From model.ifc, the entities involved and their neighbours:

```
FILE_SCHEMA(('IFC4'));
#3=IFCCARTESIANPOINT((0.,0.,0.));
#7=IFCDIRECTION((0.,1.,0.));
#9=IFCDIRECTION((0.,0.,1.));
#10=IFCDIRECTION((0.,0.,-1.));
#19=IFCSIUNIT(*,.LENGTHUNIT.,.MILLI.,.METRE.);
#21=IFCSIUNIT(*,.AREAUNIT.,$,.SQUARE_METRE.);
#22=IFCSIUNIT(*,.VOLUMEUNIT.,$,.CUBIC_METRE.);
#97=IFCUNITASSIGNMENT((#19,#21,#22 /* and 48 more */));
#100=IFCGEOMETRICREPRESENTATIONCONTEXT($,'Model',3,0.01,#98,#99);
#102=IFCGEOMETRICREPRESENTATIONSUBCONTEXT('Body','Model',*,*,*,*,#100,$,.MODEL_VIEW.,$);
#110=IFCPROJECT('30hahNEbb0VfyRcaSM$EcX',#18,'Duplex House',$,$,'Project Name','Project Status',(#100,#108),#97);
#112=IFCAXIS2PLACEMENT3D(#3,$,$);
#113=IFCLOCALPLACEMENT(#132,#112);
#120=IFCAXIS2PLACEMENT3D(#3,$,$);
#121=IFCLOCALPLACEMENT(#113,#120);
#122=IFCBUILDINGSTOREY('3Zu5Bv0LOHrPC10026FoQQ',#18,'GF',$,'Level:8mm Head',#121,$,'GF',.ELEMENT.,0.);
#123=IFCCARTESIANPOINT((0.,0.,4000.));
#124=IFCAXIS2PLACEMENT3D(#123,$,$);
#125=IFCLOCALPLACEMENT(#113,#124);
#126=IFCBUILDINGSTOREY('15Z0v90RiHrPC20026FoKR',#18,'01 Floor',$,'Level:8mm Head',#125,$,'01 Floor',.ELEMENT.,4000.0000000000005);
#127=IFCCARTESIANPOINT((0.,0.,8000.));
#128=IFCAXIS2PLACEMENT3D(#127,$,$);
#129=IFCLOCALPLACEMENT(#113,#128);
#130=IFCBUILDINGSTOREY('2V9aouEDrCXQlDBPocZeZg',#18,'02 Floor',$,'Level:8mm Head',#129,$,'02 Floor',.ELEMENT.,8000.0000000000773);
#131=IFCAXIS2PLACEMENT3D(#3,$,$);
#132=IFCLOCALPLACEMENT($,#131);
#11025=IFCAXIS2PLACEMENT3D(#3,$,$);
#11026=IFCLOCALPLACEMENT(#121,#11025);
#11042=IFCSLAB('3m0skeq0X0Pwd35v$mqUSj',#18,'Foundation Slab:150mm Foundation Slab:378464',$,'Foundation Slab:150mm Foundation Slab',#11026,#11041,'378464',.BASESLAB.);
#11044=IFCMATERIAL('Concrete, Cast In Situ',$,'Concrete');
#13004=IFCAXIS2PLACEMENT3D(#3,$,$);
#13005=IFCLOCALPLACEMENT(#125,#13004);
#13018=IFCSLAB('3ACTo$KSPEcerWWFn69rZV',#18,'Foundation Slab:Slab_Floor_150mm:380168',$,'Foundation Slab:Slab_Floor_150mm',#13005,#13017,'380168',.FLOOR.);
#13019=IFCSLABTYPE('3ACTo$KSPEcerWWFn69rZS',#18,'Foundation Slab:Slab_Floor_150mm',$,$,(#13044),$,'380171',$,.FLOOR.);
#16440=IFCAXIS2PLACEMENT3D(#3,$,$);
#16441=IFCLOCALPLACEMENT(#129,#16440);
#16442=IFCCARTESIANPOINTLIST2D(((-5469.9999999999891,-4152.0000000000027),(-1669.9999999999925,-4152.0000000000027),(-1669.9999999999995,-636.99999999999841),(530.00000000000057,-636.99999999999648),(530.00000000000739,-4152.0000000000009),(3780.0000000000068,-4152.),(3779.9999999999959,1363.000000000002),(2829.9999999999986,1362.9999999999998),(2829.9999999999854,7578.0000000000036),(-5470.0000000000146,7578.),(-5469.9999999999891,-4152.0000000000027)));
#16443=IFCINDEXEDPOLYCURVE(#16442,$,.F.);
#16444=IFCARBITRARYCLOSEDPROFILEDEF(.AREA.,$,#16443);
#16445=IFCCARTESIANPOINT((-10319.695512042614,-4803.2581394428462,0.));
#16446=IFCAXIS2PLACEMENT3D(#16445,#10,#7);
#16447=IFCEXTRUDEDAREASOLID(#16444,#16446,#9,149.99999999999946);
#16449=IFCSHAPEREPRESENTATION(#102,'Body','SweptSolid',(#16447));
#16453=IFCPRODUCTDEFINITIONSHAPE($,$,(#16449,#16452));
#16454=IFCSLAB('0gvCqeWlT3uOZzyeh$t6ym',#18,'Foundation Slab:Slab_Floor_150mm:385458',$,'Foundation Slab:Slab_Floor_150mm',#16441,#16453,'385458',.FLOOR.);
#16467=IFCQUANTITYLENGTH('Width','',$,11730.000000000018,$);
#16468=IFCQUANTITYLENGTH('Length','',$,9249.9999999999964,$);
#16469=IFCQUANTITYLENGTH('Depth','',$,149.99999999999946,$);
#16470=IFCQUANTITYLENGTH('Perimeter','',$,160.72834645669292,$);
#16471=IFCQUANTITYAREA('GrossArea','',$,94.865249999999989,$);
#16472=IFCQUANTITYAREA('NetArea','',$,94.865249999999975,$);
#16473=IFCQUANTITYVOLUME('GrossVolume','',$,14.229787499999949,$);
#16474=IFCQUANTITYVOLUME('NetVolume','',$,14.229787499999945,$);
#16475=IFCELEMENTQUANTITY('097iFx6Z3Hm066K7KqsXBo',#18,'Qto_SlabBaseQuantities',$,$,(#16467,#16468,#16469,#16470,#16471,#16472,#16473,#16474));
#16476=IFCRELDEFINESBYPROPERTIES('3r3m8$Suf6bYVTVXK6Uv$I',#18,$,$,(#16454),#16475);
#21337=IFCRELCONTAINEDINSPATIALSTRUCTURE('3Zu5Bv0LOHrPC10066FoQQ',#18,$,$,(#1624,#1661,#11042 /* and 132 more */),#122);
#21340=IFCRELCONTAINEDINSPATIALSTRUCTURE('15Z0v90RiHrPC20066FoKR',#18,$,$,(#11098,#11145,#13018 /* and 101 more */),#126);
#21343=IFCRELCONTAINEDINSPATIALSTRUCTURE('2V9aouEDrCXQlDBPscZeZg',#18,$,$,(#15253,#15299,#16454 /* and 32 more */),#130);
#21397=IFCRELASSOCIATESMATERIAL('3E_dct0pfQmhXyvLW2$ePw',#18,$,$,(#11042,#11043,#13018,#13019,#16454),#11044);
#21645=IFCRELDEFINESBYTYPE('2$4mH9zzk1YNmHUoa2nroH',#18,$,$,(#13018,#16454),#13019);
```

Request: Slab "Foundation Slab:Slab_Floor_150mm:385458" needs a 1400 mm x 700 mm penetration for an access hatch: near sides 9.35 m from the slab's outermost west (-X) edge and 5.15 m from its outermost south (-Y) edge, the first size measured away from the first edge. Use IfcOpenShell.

```python
import numpy as np
import ifcopenshell
import ifcopenshell.api.feature
import ifcopenshell.api.geometry
import ifcopenshell.api.pset
import ifcopenshell.api.root
import ifcopenshell.geom
import ifcopenshell.util.element
import ifcopenshell.util.placement
import ifcopenshell.util.representation
import ifcopenshell.util.shape
import ifcopenshell.util.unit

model = ifcopenshell.open("model.ifc")
unit_scale = ifcopenshell.util.unit.calculate_unit_scale(model)
area_scale = ifcopenshell.util.unit.calculate_unit_scale(model, "AREAUNIT")
volume_scale = ifcopenshell.util.unit.calculate_unit_scale(model, "VOLUMEUNIT")
settings = ifcopenshell.geom.settings()


def volume(element):
    """Net volume in cubic metres, openings subtracted."""
    shape = ifcopenshell.geom.create_shape(settings, element)
    return ifcopenshell.util.shape.get_volume(shape.geometry)


slab = model.by_guid("0gvCqeWlT3uOZzyeh$t6ym")
before = volume(slab)

# Extent in the slab's own axes, in metres. The edges named are its -X and -Y sides.
slab_shape = ifcopenshell.geom.create_shape(settings, slab)
vertices = ifcopenshell.util.shape.get_vertices(slab_shape.geometry)
x_min, y_min, bottom = vertices.min(axis=0)
top = vertices[:, 2].max()

opening = ifcopenshell.api.root.create_entity(model, ifc_class="IfcOpeningElement", name="Access hatch opening", predefined_type="OPENING")
context = ifcopenshell.util.representation.get_context(model, "Model", "Body", "MODEL_VIEW")
width, depth = 1.4, 0.7
outline = [(0.0, 0.0), (width, 0.0), (width, depth), (0.0, depth), (0.0, 0.0)]
# Overshoot both faces by 50 mm so the cut is clean.
shape = ifcopenshell.api.geometry.add_slab_representation(
    model, context=context, depth=top - bottom + 0.1, polyline=outline
)
ifcopenshell.api.geometry.assign_representation(model, product=opening, representation=shape)

matrix = ifcopenshell.util.placement.get_local_placement(slab.ObjectPlacement)
matrix[:, 3] = matrix @ np.append(np.array([x_min + 9.35, y_min + 5.15, bottom - 0.05]) / unit_scale, 1.0)
ifcopenshell.api.geometry.edit_object_placement(model, product=opening, matrix=matrix, is_si=False)
ifcopenshell.api.feature.add_feature(model, feature=opening, element=slab)

after = volume(slab)

# Update the slab's stored quantities.
qto = model.by_id(ifcopenshell.util.element.get_pset(slab, "Qto_SlabBaseQuantities", should_inherit=False)["id"])
ifcopenshell.api.pset.edit_qto(model, qto=qto, properties={
    "NetArea": after / (top - bottom) / area_scale,
    "NetVolume": after / volume_scale,
})

print(f"slab volume {before:.3f} -> {after:.3f} m3")

model.write("model_edited.ifc")
```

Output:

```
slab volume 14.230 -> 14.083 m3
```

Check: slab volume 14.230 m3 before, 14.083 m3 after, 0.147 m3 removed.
